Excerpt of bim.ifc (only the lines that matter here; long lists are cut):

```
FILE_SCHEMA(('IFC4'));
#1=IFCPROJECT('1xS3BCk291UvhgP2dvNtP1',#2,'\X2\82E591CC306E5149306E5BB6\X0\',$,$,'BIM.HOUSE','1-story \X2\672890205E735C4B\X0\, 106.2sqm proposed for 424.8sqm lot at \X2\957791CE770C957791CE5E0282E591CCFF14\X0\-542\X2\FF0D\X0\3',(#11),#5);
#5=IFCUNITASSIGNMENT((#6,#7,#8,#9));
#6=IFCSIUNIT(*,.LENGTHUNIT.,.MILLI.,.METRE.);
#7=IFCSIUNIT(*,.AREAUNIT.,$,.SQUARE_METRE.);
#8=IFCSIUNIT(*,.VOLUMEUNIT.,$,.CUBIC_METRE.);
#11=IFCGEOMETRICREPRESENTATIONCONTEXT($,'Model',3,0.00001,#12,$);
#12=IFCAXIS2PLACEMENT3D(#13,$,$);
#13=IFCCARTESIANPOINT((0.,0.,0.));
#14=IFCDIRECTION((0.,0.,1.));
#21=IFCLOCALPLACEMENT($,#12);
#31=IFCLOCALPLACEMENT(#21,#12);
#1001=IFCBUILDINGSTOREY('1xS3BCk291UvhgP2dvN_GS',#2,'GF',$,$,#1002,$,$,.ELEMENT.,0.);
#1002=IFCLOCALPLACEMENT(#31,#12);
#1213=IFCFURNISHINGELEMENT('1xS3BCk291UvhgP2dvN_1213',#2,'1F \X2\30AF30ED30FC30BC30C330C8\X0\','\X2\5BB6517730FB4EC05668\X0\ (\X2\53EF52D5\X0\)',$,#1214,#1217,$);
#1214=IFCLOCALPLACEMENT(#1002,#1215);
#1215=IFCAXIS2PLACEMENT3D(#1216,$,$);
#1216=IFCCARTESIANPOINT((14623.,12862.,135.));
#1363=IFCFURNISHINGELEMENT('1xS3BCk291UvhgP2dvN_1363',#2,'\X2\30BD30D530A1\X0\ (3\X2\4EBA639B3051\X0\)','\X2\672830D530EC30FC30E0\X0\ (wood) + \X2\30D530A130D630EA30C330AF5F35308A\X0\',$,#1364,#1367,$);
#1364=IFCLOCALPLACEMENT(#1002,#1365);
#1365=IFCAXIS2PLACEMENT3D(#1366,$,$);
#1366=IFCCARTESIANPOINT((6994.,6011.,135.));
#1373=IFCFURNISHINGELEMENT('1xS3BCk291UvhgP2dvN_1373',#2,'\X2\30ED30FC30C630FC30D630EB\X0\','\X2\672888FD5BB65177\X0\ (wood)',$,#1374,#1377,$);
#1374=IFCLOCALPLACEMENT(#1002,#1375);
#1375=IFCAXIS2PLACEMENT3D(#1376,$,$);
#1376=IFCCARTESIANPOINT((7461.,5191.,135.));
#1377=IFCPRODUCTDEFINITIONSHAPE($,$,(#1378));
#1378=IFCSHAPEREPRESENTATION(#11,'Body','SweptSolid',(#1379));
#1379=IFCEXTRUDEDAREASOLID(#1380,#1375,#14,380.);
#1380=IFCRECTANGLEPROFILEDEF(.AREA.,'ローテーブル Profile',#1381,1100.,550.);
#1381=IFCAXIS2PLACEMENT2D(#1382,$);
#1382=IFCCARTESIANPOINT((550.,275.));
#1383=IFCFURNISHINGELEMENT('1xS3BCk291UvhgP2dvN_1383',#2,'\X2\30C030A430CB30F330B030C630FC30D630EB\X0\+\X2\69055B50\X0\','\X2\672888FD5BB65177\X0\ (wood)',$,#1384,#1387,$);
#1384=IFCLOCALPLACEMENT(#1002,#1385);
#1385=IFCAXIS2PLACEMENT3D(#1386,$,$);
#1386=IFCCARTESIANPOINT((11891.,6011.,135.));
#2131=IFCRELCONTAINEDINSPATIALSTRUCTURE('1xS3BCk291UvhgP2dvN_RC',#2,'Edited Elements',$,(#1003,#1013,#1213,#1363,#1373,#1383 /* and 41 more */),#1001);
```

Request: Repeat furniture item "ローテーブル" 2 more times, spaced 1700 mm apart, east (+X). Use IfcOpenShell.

```python
import numpy as np
import ifcopenshell
import ifcopenshell.api.geometry
import ifcopenshell.api.root
import ifcopenshell.util.element
import ifcopenshell.util.placement

model = ifcopenshell.open("bim.ifc")


def reuse_history(source, copy):
    """copy_class also copies each property set's owner history, people and application; keep the originals."""
    for rel in copy.IsDefinedBy:
        if rel.is_a("IfcRelDefinesByProperties") and (history := rel.RelatingPropertyDefinition.OwnerHistory):
            rel.RelatingPropertyDefinition.OwnerHistory = source.OwnerHistory
            ifcopenshell.util.element.remove_deep2(model, history)


source = model.by_guid("1xS3BCk291UvhgP2dvN_1373")
base = ifcopenshell.util.placement.get_local_placement(source.ObjectPlacement)
step = np.array([1.0, 0.0, 0.0]) * 1700.0

for i in range(1, 3):
    copy = ifcopenshell.api.root.copy_class(model, product=source)
    copy.Representation = ifcopenshell.util.element.copy_deep(
        model, source.Representation, exclude=["IfcGeometricRepresentationContext", "IfcRepresentationMap"]
    )
    reuse_history(source, copy)
    matrix = base.copy()
    matrix[:3, 3] += i * step
    print("added at", matrix[:3, 3].round(3) + 0.0)
    ifcopenshell.api.geometry.edit_object_placement(model, product=copy, matrix=matrix, is_si=False)

model.write("bim_updated.ifc")
```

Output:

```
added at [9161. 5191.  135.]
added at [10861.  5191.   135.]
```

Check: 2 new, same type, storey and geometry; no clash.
